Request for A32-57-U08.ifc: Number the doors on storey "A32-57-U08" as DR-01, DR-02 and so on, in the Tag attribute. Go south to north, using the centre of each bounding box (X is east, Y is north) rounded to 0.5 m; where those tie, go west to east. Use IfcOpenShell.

First a look at what the model holds.

```python
import ifcopenshell
import ifcopenshell.util.element
import ifcopenshell.util.placement

model = ifcopenshell.open("A32-57-U08.ifc")
print(model.schema)
storey = next(s for s in model.by_type("IfcBuildingStorey") if s.Name == "A32-57-U08")
doors = [e for e in ifcopenshell.util.element.get_decomposition(storey) if e.is_a("IfcDoor")]
for e in sorted(doors, key=lambda e: e.id()):
    origin = ifcopenshell.util.placement.get_local_placement(e.ObjectPlacement)[:3, 3]
    print(e.id(), e.Tag, e.Name, origin.round(2) + 0.0, sep=" | ")
```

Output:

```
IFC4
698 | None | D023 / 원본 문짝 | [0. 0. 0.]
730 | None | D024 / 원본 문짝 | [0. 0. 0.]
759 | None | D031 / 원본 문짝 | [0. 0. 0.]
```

```python
import ifcopenshell
import ifcopenshell.geom
import ifcopenshell.util.element
import ifcopenshell.util.shape

model = ifcopenshell.open("A32-57-U08.ifc")
settings = ifcopenshell.geom.settings()
settings.set("use-world-coords", True)


def centre(element):
    shape = ifcopenshell.geom.create_shape(settings, element)
    return ifcopenshell.util.shape.get_bbox_centroid(shape.geometry)


storey = next(s for s in model.by_type("IfcBuildingStorey") if s.Name == "A32-57-U08")
doors = [e for e in ifcopenshell.util.element.get_decomposition(storey) if e.is_a("IfcDoor")]

# Insertion points can sit at a corner or the storey origin, so sort by the geometry (in metres).
centres = {e: centre(e) for e in doors}
doors.sort(key=lambda e: (round(centres[e][1] / 0.5), centres[e][0]))

for i, e in enumerate(doors, start=1):
    number = f"DR-{i:02d}"
    e.Tag = number
    print(e.id(), number)

model.write("A32-57-U08_v2.ifc")
```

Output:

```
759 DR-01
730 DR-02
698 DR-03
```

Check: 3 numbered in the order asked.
